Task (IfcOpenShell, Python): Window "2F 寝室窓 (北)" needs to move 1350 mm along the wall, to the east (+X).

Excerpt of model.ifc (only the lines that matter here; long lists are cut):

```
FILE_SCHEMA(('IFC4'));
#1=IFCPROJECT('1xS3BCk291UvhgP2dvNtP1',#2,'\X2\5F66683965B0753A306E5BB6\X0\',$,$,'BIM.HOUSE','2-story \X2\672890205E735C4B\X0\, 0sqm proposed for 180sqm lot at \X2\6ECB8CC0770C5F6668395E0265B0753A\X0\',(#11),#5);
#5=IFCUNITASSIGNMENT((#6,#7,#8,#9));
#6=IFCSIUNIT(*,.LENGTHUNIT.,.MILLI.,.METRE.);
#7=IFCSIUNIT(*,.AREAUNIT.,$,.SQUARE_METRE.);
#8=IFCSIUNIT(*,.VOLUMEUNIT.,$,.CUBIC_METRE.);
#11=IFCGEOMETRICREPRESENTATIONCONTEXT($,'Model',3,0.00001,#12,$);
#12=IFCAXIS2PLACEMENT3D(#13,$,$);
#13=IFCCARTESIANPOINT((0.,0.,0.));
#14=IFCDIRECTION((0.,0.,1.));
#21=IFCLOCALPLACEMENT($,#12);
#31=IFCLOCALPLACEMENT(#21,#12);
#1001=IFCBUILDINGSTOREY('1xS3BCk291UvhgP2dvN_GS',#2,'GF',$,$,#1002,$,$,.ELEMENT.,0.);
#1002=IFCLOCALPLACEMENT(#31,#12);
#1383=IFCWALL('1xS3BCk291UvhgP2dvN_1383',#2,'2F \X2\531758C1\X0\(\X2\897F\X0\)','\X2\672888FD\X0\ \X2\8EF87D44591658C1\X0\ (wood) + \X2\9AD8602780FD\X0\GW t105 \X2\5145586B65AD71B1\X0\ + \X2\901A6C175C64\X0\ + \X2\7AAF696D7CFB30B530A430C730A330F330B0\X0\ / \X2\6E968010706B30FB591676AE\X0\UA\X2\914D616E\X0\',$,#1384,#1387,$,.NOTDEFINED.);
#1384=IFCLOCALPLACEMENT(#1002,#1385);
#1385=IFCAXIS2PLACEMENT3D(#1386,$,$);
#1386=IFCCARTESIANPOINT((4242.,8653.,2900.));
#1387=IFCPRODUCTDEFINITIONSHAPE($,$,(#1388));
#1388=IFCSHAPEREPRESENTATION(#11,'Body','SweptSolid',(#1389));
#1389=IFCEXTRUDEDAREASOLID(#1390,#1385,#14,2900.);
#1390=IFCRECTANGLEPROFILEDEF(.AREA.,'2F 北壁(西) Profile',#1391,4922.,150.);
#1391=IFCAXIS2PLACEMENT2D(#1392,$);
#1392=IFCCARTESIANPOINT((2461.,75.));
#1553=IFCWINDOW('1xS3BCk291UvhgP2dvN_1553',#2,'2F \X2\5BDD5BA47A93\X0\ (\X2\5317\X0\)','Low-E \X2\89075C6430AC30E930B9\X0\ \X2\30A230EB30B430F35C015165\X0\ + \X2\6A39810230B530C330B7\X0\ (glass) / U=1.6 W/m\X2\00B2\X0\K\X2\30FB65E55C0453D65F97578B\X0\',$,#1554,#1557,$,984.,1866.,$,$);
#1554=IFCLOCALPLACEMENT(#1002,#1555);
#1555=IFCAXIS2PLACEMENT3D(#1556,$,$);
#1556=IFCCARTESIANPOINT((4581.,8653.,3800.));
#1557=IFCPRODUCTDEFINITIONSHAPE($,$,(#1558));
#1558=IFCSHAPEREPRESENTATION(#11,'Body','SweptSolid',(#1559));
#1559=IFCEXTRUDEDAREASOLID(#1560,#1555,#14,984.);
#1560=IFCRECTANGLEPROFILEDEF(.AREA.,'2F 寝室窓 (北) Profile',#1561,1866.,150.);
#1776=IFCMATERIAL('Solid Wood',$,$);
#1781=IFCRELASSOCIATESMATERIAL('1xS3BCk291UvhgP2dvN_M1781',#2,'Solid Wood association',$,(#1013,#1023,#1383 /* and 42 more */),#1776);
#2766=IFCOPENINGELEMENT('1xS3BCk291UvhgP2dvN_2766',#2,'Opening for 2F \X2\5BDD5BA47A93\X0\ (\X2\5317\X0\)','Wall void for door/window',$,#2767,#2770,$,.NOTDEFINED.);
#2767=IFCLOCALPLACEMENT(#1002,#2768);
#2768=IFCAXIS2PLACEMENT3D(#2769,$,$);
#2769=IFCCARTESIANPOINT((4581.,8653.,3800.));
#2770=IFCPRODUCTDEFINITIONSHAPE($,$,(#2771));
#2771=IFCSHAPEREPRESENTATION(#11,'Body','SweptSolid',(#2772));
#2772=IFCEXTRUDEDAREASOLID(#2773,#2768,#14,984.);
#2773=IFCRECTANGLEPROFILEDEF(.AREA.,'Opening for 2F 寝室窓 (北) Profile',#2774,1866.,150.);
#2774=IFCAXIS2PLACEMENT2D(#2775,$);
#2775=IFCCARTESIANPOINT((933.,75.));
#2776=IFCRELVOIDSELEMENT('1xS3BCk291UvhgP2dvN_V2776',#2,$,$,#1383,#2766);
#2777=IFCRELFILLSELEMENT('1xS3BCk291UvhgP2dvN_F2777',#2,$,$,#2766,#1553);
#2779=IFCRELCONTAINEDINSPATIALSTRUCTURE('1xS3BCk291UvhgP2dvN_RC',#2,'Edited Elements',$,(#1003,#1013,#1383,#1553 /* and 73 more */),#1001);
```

```python
import ifcopenshell
import ifcopenshell.api.geometry
import ifcopenshell.util.placement
import ifcopenshell.util.unit

model = ifcopenshell.open("model.ifc")
unit_scale = ifcopenshell.util.unit.calculate_unit_scale(model)

window = model.by_guid("1xS3BCk291UvhgP2dvN_1553")
opening = window.FillsVoids[0].RelatingOpeningElement
wall = opening.VoidsElements[0].RelatingBuildingElement

wall_matrix = ifcopenshell.util.placement.get_local_placement(wall.ObjectPlacement)
shift = wall_matrix[:3, 0] * 1.35 / unit_scale
before = ifcopenshell.util.placement.get_local_placement(window.ObjectPlacement)[:3, 3].copy()

# The window is not placed relative to its opening, so move both.
for product in (opening, window):
    matrix = ifcopenshell.util.placement.get_local_placement(product.ObjectPlacement)
    matrix[:3, 3] += shift
    ifcopenshell.api.geometry.edit_object_placement(model, product=product, matrix=matrix, is_si=False)

after = ifcopenshell.util.placement.get_local_placement(window.ObjectPlacement)[:3, 3]
print("window moved by", (after - before).round(3) + 0.0)

model.write("model_rev.ifc")
```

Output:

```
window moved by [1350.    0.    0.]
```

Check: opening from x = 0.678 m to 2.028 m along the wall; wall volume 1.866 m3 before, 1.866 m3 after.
